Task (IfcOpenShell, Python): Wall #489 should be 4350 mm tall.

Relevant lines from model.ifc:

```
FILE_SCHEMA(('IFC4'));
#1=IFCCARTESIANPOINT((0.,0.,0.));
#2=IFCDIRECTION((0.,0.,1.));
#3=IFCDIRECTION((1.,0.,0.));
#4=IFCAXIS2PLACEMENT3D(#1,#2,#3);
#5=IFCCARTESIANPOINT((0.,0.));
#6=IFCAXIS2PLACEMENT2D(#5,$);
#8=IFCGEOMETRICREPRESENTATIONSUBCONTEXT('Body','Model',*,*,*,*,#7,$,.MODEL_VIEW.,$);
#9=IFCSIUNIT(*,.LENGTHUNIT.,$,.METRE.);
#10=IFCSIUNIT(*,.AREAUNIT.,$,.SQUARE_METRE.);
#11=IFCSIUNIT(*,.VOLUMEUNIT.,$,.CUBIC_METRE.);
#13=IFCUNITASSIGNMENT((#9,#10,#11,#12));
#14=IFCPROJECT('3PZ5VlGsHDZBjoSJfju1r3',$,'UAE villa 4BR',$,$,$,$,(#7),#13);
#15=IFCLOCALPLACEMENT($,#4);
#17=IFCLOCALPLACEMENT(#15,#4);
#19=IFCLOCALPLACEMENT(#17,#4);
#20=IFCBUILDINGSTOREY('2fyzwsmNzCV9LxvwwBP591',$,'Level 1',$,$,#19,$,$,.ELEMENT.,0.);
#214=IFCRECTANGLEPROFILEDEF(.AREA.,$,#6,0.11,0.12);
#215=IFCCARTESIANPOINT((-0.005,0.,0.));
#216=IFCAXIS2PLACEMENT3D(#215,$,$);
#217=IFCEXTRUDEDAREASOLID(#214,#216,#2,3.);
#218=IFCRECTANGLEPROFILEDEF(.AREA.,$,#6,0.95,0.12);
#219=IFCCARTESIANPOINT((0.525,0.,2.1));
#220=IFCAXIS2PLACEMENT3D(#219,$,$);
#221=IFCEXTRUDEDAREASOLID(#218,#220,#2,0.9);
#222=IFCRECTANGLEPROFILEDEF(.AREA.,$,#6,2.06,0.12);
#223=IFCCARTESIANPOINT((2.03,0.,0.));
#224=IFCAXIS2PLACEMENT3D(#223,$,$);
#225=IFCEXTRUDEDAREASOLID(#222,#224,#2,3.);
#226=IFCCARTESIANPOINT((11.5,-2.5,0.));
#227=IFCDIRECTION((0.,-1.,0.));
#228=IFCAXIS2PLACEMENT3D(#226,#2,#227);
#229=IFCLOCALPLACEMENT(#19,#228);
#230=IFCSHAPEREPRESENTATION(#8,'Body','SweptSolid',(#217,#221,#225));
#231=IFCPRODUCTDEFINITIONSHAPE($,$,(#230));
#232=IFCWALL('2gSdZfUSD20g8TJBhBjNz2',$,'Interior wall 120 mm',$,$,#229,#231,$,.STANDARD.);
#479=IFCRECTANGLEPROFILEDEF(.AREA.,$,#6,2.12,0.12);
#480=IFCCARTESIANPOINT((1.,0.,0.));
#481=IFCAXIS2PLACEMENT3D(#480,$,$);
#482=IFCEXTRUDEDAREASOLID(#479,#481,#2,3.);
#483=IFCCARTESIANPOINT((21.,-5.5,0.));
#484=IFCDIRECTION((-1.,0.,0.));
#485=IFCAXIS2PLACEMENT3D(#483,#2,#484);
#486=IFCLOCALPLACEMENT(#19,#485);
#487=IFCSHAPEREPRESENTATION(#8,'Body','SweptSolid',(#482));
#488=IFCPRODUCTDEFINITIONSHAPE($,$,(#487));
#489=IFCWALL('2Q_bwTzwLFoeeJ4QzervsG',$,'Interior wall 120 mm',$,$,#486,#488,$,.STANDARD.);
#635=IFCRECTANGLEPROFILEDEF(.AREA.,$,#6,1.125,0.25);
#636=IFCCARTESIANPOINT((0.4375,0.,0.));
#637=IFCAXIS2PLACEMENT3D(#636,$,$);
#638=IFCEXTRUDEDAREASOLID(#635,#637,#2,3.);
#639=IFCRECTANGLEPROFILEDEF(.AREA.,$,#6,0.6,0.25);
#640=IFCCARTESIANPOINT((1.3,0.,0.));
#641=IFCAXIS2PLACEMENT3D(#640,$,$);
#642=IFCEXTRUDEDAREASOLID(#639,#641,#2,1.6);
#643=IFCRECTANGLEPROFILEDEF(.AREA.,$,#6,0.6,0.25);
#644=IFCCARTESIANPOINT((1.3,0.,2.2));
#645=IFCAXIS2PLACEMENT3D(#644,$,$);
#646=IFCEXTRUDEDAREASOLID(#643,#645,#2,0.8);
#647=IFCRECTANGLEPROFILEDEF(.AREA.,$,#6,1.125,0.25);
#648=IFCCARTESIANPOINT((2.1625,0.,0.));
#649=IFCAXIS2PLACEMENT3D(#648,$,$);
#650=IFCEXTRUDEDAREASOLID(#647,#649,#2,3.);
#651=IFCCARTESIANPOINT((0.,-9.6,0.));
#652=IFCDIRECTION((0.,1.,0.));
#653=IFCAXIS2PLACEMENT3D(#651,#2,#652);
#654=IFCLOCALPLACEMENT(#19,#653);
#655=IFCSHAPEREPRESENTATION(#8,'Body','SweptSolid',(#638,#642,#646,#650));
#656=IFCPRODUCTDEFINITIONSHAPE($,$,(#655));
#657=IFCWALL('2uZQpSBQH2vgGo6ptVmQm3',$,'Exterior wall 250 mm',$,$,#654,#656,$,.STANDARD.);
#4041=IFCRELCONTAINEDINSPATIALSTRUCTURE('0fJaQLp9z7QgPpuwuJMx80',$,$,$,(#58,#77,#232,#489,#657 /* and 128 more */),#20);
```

```python
import ifcopenshell
import ifcopenshell.geom
import ifcopenshell.util.representation
import ifcopenshell.util.shape

model = ifcopenshell.open("model.ifc")
settings = ifcopenshell.geom.settings()


def volume(element):
    """Net volume in cubic metres, openings subtracted."""
    shape = ifcopenshell.geom.create_shape(settings, element)
    return ifcopenshell.util.shape.get_volume(shape.geometry)


wall = model.by_id(489)
before = volume(wall)

body = ifcopenshell.util.representation.get_representation(wall, "Model", "Body")
solid = body.Items[0]
old_height = solid.Depth
solid.Depth = 4.35
after = volume(wall)

print(f"height {old_height:g} -> {solid.Depth:g}, volume {before:.3f} -> {after:.3f} m3")

model.write("model_edited.ifc")
```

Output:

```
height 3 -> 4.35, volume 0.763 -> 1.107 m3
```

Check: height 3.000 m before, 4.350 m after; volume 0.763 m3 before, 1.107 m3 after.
